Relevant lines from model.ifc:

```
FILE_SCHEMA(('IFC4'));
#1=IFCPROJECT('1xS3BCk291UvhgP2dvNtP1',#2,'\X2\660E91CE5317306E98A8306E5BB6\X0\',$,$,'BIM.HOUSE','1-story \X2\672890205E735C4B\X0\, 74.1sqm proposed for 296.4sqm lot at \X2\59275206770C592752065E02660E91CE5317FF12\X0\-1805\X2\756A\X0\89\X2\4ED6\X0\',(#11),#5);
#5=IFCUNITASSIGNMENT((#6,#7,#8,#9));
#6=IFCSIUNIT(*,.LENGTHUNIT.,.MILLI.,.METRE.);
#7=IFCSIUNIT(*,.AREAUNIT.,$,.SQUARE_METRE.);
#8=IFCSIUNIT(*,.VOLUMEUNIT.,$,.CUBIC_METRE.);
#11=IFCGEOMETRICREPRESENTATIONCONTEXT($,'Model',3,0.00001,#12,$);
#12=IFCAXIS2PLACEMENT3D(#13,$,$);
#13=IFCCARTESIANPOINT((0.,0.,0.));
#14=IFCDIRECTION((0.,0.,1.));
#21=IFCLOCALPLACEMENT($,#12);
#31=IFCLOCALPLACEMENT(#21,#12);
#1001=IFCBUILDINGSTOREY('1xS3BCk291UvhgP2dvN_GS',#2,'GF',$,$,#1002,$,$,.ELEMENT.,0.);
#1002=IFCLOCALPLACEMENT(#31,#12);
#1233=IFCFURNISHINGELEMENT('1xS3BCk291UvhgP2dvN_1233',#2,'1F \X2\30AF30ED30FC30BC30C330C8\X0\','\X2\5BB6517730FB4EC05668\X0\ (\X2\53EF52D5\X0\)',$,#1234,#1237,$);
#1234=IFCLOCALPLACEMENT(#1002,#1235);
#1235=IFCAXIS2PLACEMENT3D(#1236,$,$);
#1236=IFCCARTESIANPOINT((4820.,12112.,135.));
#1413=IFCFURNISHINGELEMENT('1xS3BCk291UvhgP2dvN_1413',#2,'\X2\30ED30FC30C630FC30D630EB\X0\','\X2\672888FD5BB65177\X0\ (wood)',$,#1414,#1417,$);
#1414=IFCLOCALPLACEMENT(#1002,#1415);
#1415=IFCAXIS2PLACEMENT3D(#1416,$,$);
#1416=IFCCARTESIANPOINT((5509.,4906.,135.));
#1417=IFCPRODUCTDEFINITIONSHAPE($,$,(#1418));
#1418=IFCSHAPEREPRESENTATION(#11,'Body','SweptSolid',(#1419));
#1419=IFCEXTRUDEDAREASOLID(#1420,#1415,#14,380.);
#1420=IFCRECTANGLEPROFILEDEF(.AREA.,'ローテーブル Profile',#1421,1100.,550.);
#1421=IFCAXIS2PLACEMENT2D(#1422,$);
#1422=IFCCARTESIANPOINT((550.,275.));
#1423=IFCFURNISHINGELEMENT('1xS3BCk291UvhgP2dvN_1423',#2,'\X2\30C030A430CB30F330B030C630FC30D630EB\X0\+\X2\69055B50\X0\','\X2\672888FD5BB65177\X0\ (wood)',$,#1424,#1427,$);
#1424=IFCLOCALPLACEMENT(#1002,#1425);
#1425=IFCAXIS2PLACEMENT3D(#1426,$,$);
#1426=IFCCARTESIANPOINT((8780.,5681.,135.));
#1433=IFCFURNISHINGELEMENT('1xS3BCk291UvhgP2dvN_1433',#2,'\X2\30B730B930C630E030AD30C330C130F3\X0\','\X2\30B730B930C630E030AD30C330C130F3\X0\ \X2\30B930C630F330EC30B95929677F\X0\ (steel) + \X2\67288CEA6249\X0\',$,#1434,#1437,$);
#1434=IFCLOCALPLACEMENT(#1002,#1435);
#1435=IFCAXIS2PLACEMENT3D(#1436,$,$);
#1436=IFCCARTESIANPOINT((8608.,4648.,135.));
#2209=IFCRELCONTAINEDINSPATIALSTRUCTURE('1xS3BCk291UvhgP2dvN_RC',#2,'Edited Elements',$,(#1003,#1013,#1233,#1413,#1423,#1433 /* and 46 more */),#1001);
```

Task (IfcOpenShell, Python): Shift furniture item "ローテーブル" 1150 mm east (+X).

```python
import ifcopenshell
import ifcopenshell.api.geometry
import ifcopenshell.util.placement

model = ifcopenshell.open("model.ifc")

item = model.by_id(1413)
matrix = ifcopenshell.util.placement.get_local_placement(item.ObjectPlacement)
matrix[0, 3] += 1150.0
ifcopenshell.api.geometry.edit_object_placement(model, product=item, matrix=matrix, is_si=False)

print(ifcopenshell.util.placement.get_local_placement(item.ObjectPlacement).round(3) + 0.0)

model.write("model-out.ifc")
```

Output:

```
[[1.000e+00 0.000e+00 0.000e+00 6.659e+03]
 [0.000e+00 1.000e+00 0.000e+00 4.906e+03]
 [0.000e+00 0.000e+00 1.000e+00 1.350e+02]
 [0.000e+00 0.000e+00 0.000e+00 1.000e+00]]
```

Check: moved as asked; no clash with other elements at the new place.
